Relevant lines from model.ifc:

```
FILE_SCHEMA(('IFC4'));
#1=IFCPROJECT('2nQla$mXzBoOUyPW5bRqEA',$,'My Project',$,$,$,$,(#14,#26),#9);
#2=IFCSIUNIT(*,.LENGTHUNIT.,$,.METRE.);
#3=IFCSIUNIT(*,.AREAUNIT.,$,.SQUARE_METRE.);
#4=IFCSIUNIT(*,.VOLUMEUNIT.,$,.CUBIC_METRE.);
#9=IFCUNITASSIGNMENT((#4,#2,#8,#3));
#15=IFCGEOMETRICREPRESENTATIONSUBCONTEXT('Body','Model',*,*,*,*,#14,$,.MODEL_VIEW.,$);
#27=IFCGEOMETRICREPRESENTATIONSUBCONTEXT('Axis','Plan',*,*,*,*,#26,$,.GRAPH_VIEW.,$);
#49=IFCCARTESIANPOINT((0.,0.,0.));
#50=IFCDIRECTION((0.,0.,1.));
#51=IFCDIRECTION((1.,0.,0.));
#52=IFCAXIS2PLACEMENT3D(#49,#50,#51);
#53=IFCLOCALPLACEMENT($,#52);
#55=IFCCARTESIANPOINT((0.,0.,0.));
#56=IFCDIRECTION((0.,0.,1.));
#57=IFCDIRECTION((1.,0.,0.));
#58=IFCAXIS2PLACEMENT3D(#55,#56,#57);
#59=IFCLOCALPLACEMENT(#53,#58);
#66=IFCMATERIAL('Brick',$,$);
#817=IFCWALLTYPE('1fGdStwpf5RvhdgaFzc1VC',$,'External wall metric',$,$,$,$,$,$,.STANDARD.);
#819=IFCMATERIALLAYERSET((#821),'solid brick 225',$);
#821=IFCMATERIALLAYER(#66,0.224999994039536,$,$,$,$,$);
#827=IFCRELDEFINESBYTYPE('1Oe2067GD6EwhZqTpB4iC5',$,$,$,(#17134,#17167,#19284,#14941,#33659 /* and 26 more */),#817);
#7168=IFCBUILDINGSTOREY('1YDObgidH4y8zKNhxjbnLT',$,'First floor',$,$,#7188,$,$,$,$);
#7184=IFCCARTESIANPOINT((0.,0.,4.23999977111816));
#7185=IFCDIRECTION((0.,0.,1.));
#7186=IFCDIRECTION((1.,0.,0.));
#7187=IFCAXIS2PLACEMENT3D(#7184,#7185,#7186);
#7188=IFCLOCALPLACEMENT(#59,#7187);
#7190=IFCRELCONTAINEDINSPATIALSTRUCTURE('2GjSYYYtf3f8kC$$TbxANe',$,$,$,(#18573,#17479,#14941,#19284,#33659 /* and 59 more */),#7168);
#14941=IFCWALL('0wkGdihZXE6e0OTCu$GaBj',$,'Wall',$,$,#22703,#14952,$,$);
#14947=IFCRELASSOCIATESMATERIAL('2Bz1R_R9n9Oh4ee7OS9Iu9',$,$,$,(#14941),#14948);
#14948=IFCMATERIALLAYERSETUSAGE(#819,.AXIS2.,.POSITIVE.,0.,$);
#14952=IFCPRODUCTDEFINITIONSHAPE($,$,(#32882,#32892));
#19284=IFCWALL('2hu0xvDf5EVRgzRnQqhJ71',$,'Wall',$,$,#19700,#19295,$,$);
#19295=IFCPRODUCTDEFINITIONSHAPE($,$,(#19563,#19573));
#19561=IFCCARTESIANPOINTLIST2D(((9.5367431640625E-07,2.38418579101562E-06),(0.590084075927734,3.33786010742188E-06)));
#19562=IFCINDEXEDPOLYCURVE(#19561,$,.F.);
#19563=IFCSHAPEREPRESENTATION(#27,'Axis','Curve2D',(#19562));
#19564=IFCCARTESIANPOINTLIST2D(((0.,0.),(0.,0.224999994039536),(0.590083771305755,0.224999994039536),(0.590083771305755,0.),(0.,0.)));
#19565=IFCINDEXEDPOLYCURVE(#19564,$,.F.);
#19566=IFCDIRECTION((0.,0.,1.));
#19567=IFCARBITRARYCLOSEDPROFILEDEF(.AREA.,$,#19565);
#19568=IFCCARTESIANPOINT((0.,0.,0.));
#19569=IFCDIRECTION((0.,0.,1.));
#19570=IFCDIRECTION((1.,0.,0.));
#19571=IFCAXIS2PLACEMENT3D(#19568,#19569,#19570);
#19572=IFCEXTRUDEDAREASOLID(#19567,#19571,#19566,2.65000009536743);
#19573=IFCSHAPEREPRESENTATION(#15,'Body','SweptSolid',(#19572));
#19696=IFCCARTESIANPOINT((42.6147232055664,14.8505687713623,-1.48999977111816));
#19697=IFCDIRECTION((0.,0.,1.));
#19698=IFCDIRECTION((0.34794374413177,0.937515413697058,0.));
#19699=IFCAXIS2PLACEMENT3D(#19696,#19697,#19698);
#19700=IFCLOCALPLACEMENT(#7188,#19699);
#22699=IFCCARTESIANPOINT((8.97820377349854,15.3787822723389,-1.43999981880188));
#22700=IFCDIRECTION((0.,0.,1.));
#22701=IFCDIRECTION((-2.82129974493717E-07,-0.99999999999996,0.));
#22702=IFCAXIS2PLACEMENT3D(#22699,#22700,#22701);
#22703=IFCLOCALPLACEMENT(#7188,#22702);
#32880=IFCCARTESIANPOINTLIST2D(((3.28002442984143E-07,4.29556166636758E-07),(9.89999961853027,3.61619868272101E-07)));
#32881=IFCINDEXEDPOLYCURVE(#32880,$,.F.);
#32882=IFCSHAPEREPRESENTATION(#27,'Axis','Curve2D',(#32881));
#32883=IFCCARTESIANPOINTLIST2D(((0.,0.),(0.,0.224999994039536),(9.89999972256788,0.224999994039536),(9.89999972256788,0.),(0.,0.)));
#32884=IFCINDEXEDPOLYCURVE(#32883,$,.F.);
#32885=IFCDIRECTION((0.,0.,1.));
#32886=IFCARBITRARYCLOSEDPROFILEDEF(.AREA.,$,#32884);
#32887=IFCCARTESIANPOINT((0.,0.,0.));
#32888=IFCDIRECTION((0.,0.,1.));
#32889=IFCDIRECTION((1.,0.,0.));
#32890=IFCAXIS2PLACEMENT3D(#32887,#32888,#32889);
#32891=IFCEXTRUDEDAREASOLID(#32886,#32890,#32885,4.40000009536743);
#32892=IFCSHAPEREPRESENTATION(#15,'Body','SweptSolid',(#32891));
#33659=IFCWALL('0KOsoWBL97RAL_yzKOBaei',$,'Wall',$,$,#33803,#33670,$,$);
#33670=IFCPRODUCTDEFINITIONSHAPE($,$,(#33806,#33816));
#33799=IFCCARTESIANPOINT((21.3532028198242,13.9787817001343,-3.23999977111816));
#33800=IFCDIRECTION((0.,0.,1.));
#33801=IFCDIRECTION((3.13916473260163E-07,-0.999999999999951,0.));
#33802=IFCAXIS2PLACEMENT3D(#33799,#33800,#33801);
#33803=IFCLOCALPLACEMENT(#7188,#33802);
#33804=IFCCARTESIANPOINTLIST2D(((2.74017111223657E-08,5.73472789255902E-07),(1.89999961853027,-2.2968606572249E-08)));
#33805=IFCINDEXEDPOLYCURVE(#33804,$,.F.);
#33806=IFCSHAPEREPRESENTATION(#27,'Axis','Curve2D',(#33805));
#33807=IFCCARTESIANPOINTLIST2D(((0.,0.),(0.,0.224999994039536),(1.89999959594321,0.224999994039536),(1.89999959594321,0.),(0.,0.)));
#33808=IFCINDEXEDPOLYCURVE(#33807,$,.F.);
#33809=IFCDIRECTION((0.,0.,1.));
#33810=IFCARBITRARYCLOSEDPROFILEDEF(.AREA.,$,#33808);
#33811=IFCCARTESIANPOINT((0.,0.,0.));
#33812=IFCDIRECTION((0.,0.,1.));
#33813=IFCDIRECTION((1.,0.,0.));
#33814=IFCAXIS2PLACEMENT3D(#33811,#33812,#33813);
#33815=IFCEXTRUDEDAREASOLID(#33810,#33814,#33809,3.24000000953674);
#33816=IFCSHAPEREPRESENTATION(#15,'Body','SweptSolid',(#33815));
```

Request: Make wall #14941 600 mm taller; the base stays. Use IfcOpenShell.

```python
import ifcopenshell
import ifcopenshell.geom
import ifcopenshell.util.representation
import ifcopenshell.util.shape
import ifcopenshell.util.unit

model = ifcopenshell.open("model.ifc")
unit_scale = ifcopenshell.util.unit.calculate_unit_scale(model)
settings = ifcopenshell.geom.settings()


def volume(element):
    """Net volume in cubic metres, openings subtracted."""
    shape = ifcopenshell.geom.create_shape(settings, element)
    return ifcopenshell.util.shape.get_volume(shape.geometry)


wall = model.by_id(14941)
before = volume(wall)

body = ifcopenshell.util.representation.get_representation(wall, "Model", "Body")
solid = body.Items[0]
old_height = solid.Depth
solid.Depth += 0.6 / unit_scale
after = volume(wall)

print(f"height {old_height:g} -> {solid.Depth:g}, volume {before:.3f} -> {after:.3f} m3")

model.write("model_edited.ifc")
```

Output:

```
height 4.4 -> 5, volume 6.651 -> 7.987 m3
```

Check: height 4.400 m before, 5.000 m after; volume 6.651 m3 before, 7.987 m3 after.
